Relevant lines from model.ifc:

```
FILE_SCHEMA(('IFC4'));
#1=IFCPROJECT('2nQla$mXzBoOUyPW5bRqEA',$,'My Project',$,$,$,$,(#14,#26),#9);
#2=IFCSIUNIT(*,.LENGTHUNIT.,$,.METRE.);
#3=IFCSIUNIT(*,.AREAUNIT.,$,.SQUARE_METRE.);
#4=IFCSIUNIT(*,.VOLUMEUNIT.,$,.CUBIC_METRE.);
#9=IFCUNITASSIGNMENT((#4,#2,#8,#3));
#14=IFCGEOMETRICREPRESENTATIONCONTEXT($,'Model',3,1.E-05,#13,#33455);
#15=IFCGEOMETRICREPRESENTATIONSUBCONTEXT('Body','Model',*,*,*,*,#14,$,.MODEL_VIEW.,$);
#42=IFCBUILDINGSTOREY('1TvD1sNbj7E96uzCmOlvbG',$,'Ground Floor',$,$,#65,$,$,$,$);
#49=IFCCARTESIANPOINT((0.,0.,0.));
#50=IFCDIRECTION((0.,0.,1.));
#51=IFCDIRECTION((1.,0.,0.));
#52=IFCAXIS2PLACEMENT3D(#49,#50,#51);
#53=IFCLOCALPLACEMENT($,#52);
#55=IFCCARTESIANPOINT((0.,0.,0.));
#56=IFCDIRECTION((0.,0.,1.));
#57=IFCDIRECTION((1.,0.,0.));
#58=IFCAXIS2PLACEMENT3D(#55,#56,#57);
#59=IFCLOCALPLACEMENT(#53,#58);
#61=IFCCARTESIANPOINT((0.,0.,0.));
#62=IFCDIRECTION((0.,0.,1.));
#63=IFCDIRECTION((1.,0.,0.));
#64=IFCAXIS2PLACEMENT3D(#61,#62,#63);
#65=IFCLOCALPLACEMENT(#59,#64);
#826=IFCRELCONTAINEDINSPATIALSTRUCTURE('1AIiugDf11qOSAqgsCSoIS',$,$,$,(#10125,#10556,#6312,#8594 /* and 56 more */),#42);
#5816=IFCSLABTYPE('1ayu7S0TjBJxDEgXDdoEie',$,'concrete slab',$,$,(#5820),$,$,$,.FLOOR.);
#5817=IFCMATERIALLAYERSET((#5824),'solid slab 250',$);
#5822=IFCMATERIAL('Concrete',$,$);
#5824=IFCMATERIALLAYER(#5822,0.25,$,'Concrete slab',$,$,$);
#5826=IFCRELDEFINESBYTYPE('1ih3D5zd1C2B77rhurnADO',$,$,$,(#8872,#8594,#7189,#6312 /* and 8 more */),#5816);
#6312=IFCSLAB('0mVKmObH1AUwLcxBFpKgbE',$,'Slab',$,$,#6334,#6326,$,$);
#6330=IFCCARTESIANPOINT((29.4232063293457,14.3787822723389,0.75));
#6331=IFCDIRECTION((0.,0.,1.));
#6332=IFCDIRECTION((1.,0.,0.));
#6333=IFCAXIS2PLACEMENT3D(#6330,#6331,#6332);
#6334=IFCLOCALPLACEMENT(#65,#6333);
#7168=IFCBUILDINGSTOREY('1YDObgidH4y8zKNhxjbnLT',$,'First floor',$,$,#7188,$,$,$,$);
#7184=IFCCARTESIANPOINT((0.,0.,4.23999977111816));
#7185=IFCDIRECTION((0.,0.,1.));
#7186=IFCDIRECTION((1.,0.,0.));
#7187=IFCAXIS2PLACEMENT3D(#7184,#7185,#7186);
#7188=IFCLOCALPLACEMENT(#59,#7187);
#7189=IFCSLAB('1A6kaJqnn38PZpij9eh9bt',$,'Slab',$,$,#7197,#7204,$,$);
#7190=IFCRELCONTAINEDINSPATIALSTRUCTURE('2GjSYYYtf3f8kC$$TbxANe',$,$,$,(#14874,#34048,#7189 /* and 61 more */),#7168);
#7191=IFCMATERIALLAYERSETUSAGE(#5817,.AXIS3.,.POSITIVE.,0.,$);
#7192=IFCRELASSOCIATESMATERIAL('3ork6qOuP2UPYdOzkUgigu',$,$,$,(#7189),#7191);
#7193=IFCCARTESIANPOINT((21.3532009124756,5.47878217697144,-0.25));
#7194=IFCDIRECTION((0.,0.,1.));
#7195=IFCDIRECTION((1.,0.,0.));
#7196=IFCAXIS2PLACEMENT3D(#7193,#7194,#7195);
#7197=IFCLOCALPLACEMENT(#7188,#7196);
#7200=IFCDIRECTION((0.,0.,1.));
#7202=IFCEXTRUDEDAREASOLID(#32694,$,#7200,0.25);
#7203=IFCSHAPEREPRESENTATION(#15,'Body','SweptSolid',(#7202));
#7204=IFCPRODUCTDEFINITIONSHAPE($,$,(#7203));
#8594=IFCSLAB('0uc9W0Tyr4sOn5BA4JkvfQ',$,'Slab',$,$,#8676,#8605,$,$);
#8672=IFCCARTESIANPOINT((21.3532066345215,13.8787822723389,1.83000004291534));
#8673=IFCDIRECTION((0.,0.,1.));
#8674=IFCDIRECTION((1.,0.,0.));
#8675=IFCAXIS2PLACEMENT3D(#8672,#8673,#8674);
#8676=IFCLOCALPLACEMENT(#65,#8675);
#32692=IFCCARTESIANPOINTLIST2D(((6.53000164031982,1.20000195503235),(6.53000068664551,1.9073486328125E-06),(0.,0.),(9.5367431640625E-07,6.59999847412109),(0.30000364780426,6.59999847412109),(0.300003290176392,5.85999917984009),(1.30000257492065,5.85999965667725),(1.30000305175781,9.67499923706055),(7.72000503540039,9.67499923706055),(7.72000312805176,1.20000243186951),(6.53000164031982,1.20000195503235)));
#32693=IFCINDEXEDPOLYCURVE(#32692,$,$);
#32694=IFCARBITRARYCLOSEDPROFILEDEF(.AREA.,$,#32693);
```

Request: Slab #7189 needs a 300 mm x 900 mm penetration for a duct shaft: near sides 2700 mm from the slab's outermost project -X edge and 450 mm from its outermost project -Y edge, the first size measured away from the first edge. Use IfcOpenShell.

```python
import numpy as np
import ifcopenshell
import ifcopenshell.api.feature
import ifcopenshell.api.geometry
import ifcopenshell.api.root
import ifcopenshell.geom
import ifcopenshell.util.placement
import ifcopenshell.util.representation
import ifcopenshell.util.shape
import ifcopenshell.util.unit

model = ifcopenshell.open("model.ifc")
unit_scale = ifcopenshell.util.unit.calculate_unit_scale(model)
settings = ifcopenshell.geom.settings()


def volume(element):
    """Net volume in cubic metres, openings subtracted."""
    shape = ifcopenshell.geom.create_shape(settings, element)
    return ifcopenshell.util.shape.get_volume(shape.geometry)


slab = model.by_guid("1A6kaJqnn38PZpij9eh9bt")
before = volume(slab)

# Extent in the slab's own axes, in metres. The edges named are its -X and -Y sides.
slab_shape = ifcopenshell.geom.create_shape(settings, slab)
vertices = ifcopenshell.util.shape.get_vertices(slab_shape.geometry)
x_min, y_min, bottom = vertices.min(axis=0)
top = vertices[:, 2].max()

opening = ifcopenshell.api.root.create_entity(model, ifc_class="IfcOpeningElement", name="Duct shaft opening", predefined_type="OPENING")
context = ifcopenshell.util.representation.get_context(model, "Model", "Body", "MODEL_VIEW")
width, depth = 0.3, 0.9
outline = [(0.0, 0.0), (width, 0.0), (width, depth), (0.0, depth), (0.0, 0.0)]
# Overshoot both faces by 50 mm so the cut is clean.
shape = ifcopenshell.api.geometry.add_slab_representation(
    model, context=context, depth=top - bottom + 0.1, polyline=outline
)
ifcopenshell.api.geometry.assign_representation(model, product=opening, representation=shape)

matrix = ifcopenshell.util.placement.get_local_placement(slab.ObjectPlacement)
matrix[:, 3] = matrix @ np.append(np.array([x_min + 2.7, y_min + 0.45, bottom - 0.05]) / unit_scale, 1.0)
ifcopenshell.api.geometry.edit_object_placement(model, product=opening, matrix=matrix, is_si=False)
ifcopenshell.api.feature.add_feature(model, feature=opening, element=slab)

after = volume(slab)

print(f"slab volume {before:.3f} -> {after:.3f} m3")

model.write("model_edited.ifc")
```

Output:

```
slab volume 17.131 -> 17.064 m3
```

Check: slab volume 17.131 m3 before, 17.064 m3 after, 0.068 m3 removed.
